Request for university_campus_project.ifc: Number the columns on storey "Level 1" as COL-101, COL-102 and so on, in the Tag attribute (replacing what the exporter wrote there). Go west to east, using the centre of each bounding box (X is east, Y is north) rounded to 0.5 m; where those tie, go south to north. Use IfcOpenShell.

First a look at what the model holds.

```python
import ifcopenshell
import ifcopenshell.util.element
import ifcopenshell.util.placement

model = ifcopenshell.open("university_campus_project.ifc")
print(model.schema)
storey = next(s for s in model.by_type("IfcBuildingStorey") if s.Name == "Level 1")
columns = [e for e in ifcopenshell.util.element.get_decomposition(storey) if e.is_a("IfcColumn")]
for e in sorted(columns, key=lambda e: e.id()):
    origin = ifcopenshell.util.placement.get_local_placement(e.ObjectPlacement)[:3, 3]
    print(e.id(), e.Tag, e.Name, origin.round(2) + 0.0, sep=" | ")
```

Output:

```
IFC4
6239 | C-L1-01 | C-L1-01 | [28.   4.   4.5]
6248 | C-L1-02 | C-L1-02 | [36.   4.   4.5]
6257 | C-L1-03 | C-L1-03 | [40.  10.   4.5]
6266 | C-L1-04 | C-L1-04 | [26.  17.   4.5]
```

```python
import ifcopenshell
import ifcopenshell.geom
import ifcopenshell.util.element
import ifcopenshell.util.shape

model = ifcopenshell.open("university_campus_project.ifc")
settings = ifcopenshell.geom.settings()
settings.set("use-world-coords", True)


def centre(element):
    shape = ifcopenshell.geom.create_shape(settings, element)
    return ifcopenshell.util.shape.get_bbox_centroid(shape.geometry)


storey = next(s for s in model.by_type("IfcBuildingStorey") if s.Name == "Level 1")
columns = [e for e in ifcopenshell.util.element.get_decomposition(storey) if e.is_a("IfcColumn")]

# Insertion points can sit at a corner or the storey origin, so sort by the geometry (in metres).
centres = {e: centre(e) for e in columns}
columns.sort(key=lambda e: (round(centres[e][0] / 0.5), centres[e][1]))

for i, e in enumerate(columns, start=1):
    number = f"COL-1{i:02d}"
    e.Tag = number
    print(e.id(), number)

model.write("university_campus_project_updated.ifc")
```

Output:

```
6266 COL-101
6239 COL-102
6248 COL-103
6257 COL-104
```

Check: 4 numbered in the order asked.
